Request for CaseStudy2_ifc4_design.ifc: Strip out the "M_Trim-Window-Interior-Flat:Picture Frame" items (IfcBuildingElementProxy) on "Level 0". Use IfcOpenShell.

First a look at what the model holds.

```python
import ifcopenshell
import ifcopenshell.util.element

model = ifcopenshell.open("CaseStudy2_ifc4_design.ifc")
print(model.schema)
storey = next(s for s in model.by_type("IfcBuildingStorey") if s.Name == "Level 0")
proxies = [e for e in ifcopenshell.util.element.get_decomposition(storey) if e.is_a("IfcBuildingElementProxy")]
seen = {}
for e in proxies:
    element_type = ifcopenshell.util.element.get_type(e)
    name = element_type.Name if element_type not in (None, e) else None
    seen[name] = seen.get(name, 0) + 1
for name, count in sorted(seen.items(), key=str):
    print(count, "x", name)
```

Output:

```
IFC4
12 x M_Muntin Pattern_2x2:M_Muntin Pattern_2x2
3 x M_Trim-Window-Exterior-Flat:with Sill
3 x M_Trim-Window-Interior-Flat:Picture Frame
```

```python
import ifcopenshell
import ifcopenshell.api.root
import ifcopenshell.util.element

model = ifcopenshell.open("CaseStudy2_ifc4_design.ifc")

storey = next(s for s in model.by_type("IfcBuildingStorey") if s.Name == "Level 0")
proxies = [e for e in ifcopenshell.util.element.get_decomposition(storey) if e.is_a("IfcBuildingElementProxy")]
targets = [e for e in proxies if (t := ifcopenshell.util.element.get_type(e)) not in (None, e) and t.Name == "M_Trim-Window-Interior-Flat:Picture Frame"]

for e in targets:
    ifcopenshell.api.root.remove_product(model, product=e)
print(len(targets), "removed")

model.write("CaseStudy2_ifc4_design-out.ifc")
```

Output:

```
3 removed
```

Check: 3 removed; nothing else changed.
